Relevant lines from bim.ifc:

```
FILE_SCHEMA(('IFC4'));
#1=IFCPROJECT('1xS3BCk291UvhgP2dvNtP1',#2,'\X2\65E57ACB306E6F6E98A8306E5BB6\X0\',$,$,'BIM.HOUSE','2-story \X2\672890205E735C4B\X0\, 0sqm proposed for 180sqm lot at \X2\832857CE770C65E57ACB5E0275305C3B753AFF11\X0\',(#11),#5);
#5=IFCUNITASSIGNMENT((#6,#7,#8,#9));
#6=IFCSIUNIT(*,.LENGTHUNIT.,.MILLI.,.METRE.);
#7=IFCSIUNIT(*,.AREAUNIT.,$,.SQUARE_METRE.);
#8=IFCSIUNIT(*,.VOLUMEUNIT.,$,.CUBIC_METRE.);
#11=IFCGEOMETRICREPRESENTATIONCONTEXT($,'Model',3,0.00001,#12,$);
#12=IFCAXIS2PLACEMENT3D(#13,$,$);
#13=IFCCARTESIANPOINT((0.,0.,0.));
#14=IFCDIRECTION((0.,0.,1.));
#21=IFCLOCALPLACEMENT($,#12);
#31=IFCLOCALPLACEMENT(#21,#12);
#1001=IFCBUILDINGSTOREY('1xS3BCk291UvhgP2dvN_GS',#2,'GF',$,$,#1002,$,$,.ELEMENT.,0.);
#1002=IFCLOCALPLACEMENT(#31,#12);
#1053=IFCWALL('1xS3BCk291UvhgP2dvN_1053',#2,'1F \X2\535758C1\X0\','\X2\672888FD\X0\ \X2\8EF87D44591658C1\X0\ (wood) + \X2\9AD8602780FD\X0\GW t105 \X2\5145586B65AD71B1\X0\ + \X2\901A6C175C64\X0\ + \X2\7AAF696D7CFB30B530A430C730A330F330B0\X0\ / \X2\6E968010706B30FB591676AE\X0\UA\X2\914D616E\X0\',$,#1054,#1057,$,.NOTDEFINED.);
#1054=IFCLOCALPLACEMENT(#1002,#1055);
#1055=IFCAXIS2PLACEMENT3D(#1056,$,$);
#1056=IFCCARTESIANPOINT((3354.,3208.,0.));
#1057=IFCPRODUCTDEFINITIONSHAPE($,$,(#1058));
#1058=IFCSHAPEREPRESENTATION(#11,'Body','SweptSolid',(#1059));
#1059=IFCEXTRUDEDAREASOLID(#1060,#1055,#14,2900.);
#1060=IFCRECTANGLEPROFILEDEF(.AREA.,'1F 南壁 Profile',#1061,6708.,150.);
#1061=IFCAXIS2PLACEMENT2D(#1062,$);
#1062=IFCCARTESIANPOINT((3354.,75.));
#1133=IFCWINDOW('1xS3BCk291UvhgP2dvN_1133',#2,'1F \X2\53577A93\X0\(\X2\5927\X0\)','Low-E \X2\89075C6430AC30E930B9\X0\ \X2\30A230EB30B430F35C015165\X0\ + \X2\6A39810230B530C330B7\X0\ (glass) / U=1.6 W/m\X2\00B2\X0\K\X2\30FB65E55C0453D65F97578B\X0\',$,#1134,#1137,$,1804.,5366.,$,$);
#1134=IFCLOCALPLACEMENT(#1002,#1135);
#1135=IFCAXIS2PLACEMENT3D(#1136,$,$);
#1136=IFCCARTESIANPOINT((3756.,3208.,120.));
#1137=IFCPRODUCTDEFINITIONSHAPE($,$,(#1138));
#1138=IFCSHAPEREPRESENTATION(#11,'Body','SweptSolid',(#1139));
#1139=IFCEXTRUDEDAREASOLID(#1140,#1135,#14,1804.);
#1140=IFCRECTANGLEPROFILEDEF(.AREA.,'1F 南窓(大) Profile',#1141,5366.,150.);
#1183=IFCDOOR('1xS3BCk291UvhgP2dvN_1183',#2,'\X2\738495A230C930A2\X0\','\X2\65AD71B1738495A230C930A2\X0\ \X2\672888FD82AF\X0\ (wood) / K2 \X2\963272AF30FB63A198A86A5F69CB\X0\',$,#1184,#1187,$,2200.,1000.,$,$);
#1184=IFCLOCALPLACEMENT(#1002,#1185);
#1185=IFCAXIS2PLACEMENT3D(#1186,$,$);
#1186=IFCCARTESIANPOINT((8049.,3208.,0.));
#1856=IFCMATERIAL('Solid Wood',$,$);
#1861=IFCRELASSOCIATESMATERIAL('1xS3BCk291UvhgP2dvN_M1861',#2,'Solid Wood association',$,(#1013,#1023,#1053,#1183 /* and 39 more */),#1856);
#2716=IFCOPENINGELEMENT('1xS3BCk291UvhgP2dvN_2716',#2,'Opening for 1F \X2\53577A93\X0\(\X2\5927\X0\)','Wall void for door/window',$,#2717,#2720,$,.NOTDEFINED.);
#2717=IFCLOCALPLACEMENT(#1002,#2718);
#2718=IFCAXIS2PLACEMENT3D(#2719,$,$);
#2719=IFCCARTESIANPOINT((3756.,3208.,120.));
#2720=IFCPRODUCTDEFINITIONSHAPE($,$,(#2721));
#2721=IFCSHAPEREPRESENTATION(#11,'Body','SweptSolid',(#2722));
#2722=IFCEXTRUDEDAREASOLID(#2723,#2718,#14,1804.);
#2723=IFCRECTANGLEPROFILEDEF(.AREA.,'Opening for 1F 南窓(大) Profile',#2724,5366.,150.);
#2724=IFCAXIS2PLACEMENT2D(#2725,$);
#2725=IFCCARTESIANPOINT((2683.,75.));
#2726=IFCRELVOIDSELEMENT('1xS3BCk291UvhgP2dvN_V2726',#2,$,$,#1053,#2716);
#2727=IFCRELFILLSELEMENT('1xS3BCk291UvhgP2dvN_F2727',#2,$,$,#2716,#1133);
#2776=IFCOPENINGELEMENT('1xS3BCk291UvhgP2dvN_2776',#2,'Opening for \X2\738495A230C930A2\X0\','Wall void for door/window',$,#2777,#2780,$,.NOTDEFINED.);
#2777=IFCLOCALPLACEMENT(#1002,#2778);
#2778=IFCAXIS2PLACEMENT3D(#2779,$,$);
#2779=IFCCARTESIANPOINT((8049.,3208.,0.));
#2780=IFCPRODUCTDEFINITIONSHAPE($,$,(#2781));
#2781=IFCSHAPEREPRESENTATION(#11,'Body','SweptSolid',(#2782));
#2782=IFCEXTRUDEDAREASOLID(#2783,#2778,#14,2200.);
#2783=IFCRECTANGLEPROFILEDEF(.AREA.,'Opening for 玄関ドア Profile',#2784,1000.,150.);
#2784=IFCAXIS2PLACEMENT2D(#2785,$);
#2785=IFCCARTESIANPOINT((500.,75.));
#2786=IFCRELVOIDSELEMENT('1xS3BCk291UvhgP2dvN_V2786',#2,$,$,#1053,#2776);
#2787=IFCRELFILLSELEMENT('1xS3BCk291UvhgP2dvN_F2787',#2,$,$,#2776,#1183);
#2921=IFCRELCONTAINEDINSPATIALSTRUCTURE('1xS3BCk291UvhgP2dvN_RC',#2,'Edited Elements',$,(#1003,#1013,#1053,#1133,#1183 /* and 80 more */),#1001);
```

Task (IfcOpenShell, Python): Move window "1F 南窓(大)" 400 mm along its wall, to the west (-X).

```python
import ifcopenshell
import ifcopenshell.api.geometry
import ifcopenshell.util.placement
import ifcopenshell.util.unit

model = ifcopenshell.open("bim.ifc")
unit_scale = ifcopenshell.util.unit.calculate_unit_scale(model)

window = model.by_guid("1xS3BCk291UvhgP2dvN_1133")
opening = window.FillsVoids[0].RelatingOpeningElement
wall = opening.VoidsElements[0].RelatingBuildingElement

wall_matrix = ifcopenshell.util.placement.get_local_placement(wall.ObjectPlacement)
shift = wall_matrix[:3, 0] * -0.4 / unit_scale
before = ifcopenshell.util.placement.get_local_placement(window.ObjectPlacement)[:3, 3].copy()

# The window is not placed relative to its opening, so move both.
for product in (opening, window):
    matrix = ifcopenshell.util.placement.get_local_placement(product.ObjectPlacement)
    matrix[:3, 3] += shift
    ifcopenshell.api.geometry.edit_object_placement(model, product=product, matrix=matrix, is_si=False)

after = ifcopenshell.util.placement.get_local_placement(window.ObjectPlacement)[:3, 3]
print("window moved by", (after - before).round(3) + 0.0)

model.write("bim-out.ifc")
```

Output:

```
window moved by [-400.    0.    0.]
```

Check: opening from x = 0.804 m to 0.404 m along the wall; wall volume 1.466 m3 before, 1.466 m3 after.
